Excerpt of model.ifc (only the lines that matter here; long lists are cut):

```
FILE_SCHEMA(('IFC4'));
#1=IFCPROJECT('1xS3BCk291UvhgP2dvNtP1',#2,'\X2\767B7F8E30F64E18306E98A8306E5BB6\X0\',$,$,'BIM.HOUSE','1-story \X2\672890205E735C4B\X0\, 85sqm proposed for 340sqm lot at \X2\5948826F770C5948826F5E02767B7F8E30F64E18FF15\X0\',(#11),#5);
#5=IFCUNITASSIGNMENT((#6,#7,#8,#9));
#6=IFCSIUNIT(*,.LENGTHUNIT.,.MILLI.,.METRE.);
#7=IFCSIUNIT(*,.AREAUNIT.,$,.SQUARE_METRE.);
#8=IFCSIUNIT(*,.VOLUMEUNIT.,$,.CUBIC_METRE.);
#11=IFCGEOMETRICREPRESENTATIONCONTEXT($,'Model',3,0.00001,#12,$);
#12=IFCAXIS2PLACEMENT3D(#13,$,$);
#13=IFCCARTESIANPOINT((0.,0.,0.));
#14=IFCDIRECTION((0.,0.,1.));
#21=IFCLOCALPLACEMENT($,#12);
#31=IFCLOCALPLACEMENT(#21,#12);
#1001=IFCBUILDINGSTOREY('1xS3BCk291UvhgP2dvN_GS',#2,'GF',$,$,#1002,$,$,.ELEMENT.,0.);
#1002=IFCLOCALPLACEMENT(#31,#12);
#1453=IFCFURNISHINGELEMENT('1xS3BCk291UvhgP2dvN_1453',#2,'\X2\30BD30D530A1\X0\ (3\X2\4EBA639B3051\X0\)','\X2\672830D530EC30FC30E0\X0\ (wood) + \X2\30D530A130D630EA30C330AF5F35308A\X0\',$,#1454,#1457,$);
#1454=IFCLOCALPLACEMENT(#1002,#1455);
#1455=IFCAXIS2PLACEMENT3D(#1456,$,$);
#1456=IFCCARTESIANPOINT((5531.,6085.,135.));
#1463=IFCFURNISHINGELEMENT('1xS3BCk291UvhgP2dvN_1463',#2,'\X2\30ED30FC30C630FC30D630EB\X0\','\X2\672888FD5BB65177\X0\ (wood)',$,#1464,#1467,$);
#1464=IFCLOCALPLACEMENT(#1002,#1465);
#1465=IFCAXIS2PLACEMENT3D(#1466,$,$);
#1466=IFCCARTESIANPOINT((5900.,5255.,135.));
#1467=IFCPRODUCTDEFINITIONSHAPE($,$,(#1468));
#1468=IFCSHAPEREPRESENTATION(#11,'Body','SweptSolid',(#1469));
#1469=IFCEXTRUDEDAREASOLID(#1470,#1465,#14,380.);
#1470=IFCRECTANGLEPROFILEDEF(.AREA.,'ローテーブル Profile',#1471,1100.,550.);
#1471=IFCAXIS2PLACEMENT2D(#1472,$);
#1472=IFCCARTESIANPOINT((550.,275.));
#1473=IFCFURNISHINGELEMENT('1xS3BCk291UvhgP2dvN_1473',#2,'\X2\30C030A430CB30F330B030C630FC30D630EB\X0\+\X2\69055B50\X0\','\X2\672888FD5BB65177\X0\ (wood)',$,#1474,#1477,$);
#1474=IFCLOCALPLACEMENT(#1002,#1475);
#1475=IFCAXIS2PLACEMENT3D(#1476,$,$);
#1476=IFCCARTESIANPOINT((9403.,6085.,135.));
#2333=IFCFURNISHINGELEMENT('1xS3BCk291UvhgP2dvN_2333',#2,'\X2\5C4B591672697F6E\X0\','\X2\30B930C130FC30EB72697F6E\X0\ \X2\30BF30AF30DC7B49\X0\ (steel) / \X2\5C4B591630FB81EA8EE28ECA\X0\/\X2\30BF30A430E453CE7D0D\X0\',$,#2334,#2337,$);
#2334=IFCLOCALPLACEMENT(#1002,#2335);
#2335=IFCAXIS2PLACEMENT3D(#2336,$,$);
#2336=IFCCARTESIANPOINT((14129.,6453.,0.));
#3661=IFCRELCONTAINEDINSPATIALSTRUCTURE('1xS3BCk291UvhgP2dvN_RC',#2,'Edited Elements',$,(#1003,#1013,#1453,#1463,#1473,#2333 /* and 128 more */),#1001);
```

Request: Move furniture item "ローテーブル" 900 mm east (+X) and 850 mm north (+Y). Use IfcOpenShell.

```python
import ifcopenshell
import ifcopenshell.api.geometry
import ifcopenshell.util.placement
import ifcopenshell.util.unit

model = ifcopenshell.open("model.ifc")
unit_scale = ifcopenshell.util.unit.calculate_unit_scale(model)

item = model.by_id(1463)
matrix = ifcopenshell.util.placement.get_local_placement(item.ObjectPlacement)
matrix[0, 3] += 0.9 / unit_scale
matrix[1, 3] += 0.85 / unit_scale
ifcopenshell.api.geometry.edit_object_placement(model, product=item, matrix=matrix, is_si=False)

print(ifcopenshell.util.placement.get_local_placement(item.ObjectPlacement).round(3) + 0.0)

model.write("model_v2.ifc")
```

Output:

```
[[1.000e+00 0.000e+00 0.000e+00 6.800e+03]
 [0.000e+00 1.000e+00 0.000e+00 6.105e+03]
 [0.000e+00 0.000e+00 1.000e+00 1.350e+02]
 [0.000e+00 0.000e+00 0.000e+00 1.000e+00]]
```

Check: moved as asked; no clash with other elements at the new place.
